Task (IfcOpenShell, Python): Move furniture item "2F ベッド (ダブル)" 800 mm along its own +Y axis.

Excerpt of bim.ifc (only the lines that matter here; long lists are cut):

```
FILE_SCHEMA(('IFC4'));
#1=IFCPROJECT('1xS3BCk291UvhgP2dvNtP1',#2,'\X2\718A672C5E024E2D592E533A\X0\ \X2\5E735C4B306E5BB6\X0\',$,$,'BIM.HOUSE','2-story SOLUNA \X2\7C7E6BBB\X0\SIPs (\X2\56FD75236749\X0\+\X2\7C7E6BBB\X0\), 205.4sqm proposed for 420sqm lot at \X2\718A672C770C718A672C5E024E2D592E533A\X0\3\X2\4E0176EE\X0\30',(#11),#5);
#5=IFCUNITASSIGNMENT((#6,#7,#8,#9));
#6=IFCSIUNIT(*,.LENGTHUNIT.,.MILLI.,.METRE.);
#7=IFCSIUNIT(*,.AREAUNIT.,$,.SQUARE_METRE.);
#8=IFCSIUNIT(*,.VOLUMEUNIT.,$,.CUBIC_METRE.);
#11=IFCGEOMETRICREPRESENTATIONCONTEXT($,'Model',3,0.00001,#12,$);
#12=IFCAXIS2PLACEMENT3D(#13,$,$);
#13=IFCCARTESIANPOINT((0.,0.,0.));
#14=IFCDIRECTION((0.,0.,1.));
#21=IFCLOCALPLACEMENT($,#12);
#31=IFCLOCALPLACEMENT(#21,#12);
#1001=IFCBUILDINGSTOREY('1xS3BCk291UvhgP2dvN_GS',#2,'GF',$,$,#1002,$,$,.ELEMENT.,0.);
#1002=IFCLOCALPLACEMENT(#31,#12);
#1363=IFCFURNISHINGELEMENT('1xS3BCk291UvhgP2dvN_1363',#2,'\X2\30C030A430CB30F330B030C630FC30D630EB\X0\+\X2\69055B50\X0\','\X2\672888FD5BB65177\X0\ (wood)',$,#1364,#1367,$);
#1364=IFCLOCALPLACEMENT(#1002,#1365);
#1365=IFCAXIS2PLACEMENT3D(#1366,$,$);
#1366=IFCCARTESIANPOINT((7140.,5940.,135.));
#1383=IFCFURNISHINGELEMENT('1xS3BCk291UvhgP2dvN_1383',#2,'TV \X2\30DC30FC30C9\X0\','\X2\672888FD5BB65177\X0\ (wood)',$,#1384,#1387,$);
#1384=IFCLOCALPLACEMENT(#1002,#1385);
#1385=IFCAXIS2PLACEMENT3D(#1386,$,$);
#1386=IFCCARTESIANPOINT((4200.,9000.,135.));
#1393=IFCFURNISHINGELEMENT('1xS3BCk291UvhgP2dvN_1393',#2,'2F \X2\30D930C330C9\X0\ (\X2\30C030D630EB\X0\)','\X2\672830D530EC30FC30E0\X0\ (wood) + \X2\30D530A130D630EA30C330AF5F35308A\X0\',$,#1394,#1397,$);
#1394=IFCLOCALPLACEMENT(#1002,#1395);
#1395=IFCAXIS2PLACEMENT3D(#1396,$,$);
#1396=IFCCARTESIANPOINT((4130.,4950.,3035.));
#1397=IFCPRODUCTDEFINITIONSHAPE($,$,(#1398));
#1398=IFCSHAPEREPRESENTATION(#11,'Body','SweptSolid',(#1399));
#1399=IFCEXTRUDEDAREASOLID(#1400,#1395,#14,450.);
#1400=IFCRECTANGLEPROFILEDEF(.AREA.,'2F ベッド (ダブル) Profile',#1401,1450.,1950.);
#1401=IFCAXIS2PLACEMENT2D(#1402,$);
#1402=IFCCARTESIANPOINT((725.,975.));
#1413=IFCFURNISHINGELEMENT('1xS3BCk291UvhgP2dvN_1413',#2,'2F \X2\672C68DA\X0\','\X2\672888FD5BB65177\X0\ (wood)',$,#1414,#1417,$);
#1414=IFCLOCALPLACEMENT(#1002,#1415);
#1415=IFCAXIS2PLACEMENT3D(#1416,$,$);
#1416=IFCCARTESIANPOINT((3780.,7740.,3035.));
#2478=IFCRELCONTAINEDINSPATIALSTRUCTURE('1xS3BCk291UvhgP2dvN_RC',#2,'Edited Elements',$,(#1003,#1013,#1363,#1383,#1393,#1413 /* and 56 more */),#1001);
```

```python
import ifcopenshell
import ifcopenshell.api.geometry
import ifcopenshell.util.placement

model = ifcopenshell.open("bim.ifc")

item = model.by_id(1393)
matrix = ifcopenshell.util.placement.get_local_placement(item.ObjectPlacement)
matrix[:3, 3] += matrix[:3, 1] * 800.0
ifcopenshell.api.geometry.edit_object_placement(model, product=item, matrix=matrix, is_si=False)

print(ifcopenshell.util.placement.get_local_placement(item.ObjectPlacement).round(3) + 0.0)

model.write("bim-out.ifc")
```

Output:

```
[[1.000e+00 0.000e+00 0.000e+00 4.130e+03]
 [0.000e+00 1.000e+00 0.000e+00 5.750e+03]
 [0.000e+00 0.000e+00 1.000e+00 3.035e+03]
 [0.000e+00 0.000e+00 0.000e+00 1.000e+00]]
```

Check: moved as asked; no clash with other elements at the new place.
